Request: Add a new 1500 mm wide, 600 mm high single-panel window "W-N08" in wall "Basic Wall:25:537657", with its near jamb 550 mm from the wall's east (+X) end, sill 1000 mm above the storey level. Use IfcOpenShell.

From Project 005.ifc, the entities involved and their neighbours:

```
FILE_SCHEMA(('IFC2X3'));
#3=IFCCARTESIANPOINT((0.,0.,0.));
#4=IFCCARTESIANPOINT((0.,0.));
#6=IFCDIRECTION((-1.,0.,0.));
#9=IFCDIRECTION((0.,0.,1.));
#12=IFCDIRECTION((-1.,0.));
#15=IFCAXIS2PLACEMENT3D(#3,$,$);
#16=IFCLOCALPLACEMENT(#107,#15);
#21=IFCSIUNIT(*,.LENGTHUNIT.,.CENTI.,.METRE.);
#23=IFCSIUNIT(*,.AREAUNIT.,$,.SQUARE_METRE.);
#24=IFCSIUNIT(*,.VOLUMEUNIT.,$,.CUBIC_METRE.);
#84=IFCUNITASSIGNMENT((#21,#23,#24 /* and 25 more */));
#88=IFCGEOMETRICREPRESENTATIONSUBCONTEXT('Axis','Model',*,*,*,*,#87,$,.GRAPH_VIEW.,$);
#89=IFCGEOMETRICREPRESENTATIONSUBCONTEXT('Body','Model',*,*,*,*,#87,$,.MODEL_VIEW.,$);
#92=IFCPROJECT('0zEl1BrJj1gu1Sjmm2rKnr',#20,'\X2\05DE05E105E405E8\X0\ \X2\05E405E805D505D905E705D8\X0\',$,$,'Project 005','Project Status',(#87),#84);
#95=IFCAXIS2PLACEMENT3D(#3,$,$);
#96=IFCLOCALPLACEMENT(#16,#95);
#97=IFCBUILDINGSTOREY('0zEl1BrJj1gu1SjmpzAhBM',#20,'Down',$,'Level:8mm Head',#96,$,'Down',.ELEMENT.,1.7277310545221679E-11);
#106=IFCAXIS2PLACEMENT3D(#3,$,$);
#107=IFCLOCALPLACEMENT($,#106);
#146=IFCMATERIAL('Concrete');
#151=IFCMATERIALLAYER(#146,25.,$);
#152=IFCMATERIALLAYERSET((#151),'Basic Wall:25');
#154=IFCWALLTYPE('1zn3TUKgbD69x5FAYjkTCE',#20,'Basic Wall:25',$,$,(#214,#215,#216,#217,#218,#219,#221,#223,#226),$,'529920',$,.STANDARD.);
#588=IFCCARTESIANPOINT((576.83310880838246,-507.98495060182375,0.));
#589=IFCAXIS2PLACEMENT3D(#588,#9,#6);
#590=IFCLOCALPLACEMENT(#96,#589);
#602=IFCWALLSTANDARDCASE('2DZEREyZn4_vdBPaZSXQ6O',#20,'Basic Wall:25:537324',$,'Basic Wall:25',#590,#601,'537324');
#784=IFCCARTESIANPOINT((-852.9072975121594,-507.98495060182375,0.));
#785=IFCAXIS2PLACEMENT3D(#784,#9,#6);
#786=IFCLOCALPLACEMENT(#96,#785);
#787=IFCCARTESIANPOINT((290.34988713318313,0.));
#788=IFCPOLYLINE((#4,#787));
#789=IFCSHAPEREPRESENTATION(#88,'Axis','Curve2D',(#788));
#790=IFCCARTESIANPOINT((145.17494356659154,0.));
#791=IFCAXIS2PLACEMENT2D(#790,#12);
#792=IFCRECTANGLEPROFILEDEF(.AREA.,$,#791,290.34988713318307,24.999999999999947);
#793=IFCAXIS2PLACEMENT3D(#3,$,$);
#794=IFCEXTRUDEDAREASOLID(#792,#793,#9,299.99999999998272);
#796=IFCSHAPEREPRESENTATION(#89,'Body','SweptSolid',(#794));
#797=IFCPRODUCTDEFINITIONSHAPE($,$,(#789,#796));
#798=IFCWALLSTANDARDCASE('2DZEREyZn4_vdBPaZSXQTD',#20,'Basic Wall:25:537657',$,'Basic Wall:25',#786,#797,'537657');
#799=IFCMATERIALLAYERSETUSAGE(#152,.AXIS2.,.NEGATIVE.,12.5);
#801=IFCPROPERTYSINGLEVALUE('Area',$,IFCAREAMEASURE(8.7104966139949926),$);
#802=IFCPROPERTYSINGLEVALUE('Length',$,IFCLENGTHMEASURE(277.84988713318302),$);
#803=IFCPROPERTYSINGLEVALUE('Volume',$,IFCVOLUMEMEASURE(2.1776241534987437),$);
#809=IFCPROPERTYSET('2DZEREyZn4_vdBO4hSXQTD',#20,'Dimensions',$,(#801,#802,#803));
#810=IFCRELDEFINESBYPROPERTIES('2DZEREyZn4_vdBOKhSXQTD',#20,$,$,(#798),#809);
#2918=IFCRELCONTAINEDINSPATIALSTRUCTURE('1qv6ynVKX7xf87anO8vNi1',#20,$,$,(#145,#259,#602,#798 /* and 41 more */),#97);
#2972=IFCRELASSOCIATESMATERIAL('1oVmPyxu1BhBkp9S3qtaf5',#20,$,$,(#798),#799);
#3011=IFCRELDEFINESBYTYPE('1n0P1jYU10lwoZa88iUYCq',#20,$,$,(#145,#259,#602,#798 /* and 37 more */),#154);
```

```python
import numpy as np
import ifcopenshell
import ifcopenshell.api.feature
import ifcopenshell.api.geometry
import ifcopenshell.api.pset
import ifcopenshell.api.root
import ifcopenshell.api.spatial
import ifcopenshell.api.type
import ifcopenshell.geom
import ifcopenshell.util.element
import ifcopenshell.util.placement
import ifcopenshell.util.representation
import ifcopenshell.util.shape
import ifcopenshell.util.unit

model = ifcopenshell.open("Project 005.ifc")
unit_scale = ifcopenshell.util.unit.calculate_unit_scale(model)
area_scale = ifcopenshell.util.unit.calculate_unit_scale(model, "AREAUNIT")
volume_scale = ifcopenshell.util.unit.calculate_unit_scale(model, "VOLUMEUNIT")
settings = ifcopenshell.geom.settings()


def volume(element):
    """Net volume in cubic metres, openings subtracted."""
    shape = ifcopenshell.geom.create_shape(settings, element)
    return ifcopenshell.util.shape.get_volume(shape.geometry)


wall = model.by_guid("2DZEREyZn4_vdBPaZSXQTD")
storey = ifcopenshell.util.element.get_container(wall, ifc_class="IfcBuildingStorey")
context = ifcopenshell.util.representation.get_context(model, "Model", "Body", "MODEL_VIEW")
before = volume(wall)

width, height, from_end, sill = 1.5, 0.6, 0.55, 1  # metres

# The wall runs along its own X axis, and the end named is its -X end.
wall_shape = ifcopenshell.geom.create_shape(settings, wall)
x, y, z = ifcopenshell.util.shape.get_vertices(wall_shape.geometry).T
start = x.min() + from_end
face, thickness = float(y.min()), float(y.max() - y.min())
wall_matrix = ifcopenshell.util.placement.get_local_placement(wall.ObjectPlacement)
level = ifcopenshell.util.placement.get_local_placement(storey.ObjectPlacement)[2, 3]


def in_wall(x, y):
    """Placement at x, y metres in the wall's axes, at sill height."""
    matrix = wall_matrix.copy()
    matrix[:, 3] = wall_matrix @ np.array([x / unit_scale, y / unit_scale, 0.0, 1.0])
    matrix[2, 3] = level + sill / unit_scale
    return matrix


# Opening: a box that overshoots both wall faces by 50 mm.
opening = ifcopenshell.api.root.create_entity(model, ifc_class="IfcOpeningElement")
box = ifcopenshell.api.geometry.add_wall_representation(
    model, context=context, length=width, height=height, thickness=thickness + 0.1
)
ifcopenshell.api.geometry.assign_representation(model, product=opening, representation=box)
ifcopenshell.api.geometry.edit_object_placement(model, product=opening, matrix=in_wall(start, face - 0.05), is_si=False)
ifcopenshell.api.feature.add_feature(model, feature=opening, element=wall)

window = ifcopenshell.api.root.create_entity(model, ifc_class="IfcWindow", name="W-N08")
window.OverallWidth, window.OverallHeight = width / unit_scale, height / unit_scale
body = ifcopenshell.api.geometry.add_window_representation(
    model,
    context=context,
    overall_width=window.OverallWidth,
    overall_height=window.OverallHeight,
    partition_type="SINGLE_PANEL",
)
ifcopenshell.api.geometry.assign_representation(model, product=window, representation=body)
ifcopenshell.api.spatial.assign_container(model, products=[window], relating_structure=storey)
fills = ifcopenshell.api.feature.add_filling(model, opening=opening, element=window)
fills.OwnerHistory = window.OwnerHistory  # required in IFC2X3

# IFC2X3 keeps the operation on the window style.
style = ifcopenshell.api.root.create_entity(model, ifc_class="IfcWindowStyle", name="W-N08")
style.OperationType, style.ConstructionType = "SINGLE_PANEL", "NOTDEFINED"
style.ParameterTakesPrecedence = style.Sizeable = False
ifcopenshell.api.type.assign_type(model, related_objects=[window], relating_type=style)

# Centre the window in the wall's thickness.
ifcopenshell.api.geometry.edit_object_placement(model, product=window, matrix=in_wall(start, face), is_si=False)
window_shape = ifcopenshell.geom.create_shape(settings, window)
depth = ifcopenshell.util.shape.get_vertices(window_shape.geometry)[:, 1]
offset = face + thickness / 2 - (depth.min() + depth.max()) / 2
ifcopenshell.api.geometry.edit_object_placement(model, product=window, matrix=in_wall(start, offset), is_si=False)

after = volume(wall)

# Update the wall's stored quantities.
pset = model.by_id(ifcopenshell.util.element.get_pset(wall, "Dimensions", should_inherit=False)["id"])
ifcopenshell.api.pset.edit_pset(model, pset=pset, properties={
    "Area": model.create_entity("IfcAreaMeasure", after / thickness / area_scale),
    "Volume": model.create_entity("IfcVolumeMeasure", after / volume_scale),
})

print(f"wall volume {before:.3f} -> {after:.3f} m3")

model.write("Project 005_rev.ifc")
```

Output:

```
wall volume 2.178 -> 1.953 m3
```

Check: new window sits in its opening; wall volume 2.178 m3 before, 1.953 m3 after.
